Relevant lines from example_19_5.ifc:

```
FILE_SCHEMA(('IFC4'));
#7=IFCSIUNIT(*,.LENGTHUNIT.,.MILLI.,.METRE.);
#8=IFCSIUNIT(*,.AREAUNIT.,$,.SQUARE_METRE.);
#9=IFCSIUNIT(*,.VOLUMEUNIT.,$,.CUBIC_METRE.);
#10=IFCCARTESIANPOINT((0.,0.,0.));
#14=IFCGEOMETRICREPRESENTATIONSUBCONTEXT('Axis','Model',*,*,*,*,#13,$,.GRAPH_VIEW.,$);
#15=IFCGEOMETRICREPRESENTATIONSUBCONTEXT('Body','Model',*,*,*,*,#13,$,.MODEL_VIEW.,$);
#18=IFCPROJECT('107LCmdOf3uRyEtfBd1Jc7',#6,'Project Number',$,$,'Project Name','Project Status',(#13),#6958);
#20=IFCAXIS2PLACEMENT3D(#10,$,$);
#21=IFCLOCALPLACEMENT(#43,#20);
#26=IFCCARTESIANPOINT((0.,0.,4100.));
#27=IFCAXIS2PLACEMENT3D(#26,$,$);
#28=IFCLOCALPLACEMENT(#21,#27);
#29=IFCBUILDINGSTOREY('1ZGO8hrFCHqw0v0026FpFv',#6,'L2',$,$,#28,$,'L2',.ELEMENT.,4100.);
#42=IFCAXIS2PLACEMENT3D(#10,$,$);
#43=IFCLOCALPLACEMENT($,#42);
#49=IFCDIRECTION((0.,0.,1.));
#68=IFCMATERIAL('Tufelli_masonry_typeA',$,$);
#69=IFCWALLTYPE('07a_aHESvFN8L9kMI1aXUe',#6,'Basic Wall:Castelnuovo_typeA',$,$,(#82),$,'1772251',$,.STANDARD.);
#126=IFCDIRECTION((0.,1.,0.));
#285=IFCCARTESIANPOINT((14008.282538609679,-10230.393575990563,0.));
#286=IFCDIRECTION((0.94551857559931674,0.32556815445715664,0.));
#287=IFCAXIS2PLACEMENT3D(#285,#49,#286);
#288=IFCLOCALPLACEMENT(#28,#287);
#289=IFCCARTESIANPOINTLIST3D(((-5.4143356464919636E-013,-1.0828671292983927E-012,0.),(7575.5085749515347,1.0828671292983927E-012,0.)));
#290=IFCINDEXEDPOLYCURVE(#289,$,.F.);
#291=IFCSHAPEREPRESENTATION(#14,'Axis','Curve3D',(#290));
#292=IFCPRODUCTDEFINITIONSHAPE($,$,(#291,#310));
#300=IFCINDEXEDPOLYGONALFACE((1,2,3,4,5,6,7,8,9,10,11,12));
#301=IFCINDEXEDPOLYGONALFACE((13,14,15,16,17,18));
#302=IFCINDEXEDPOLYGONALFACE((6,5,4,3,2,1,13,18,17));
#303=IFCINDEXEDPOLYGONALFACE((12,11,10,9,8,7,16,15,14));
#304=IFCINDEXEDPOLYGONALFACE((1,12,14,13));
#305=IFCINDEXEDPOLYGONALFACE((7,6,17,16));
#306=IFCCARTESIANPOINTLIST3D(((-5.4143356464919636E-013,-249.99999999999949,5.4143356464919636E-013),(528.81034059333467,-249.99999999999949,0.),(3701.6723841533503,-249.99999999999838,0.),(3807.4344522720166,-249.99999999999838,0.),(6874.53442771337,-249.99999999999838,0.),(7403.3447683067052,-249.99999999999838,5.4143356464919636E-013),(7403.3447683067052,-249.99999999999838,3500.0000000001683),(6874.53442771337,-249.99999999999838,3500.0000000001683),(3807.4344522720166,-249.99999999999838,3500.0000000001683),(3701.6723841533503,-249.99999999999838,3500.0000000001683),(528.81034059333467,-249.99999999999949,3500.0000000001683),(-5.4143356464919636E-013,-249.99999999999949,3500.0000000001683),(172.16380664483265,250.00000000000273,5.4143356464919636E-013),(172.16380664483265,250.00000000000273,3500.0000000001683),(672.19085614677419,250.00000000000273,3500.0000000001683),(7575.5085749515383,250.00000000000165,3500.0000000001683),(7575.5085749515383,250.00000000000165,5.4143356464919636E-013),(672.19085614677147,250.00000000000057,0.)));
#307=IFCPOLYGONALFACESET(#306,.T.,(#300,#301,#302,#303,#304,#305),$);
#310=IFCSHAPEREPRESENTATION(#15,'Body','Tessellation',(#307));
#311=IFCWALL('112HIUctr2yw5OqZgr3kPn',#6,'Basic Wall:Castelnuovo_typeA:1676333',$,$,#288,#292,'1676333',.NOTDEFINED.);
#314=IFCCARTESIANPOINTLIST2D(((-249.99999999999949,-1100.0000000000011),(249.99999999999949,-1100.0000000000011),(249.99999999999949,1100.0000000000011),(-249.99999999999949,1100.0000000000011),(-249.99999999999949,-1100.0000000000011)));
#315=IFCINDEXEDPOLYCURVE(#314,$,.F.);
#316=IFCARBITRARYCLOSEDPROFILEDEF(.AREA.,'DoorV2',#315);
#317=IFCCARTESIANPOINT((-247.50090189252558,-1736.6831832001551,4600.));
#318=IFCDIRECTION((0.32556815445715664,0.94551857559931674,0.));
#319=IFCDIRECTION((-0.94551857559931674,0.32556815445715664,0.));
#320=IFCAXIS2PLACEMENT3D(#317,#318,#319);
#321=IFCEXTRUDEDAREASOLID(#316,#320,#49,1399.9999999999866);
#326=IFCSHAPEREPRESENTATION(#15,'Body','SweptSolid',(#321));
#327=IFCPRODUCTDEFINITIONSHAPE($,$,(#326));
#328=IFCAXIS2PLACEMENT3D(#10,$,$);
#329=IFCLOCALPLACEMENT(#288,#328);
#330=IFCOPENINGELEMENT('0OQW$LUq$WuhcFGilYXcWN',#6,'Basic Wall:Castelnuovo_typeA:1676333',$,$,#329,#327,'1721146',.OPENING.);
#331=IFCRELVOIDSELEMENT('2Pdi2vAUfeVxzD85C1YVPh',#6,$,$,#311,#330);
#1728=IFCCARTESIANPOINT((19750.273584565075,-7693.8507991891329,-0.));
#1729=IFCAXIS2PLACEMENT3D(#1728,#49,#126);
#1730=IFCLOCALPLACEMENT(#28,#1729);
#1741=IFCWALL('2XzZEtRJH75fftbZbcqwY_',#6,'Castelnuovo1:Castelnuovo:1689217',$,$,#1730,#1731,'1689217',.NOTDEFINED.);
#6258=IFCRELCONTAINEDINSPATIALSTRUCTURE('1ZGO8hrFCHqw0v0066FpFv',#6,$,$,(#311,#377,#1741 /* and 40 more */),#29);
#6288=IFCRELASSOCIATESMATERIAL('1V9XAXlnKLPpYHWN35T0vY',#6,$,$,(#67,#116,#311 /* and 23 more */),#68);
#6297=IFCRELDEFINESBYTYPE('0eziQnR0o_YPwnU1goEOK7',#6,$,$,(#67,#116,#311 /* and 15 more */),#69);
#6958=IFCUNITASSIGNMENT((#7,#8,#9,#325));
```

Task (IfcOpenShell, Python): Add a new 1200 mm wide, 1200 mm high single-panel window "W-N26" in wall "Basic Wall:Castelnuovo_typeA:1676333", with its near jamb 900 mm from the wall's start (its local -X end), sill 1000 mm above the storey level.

```python
import numpy as np
import ifcopenshell
import ifcopenshell.api.feature
import ifcopenshell.api.geometry
import ifcopenshell.api.root
import ifcopenshell.api.spatial
import ifcopenshell.geom
import ifcopenshell.util.element
import ifcopenshell.util.placement
import ifcopenshell.util.representation
import ifcopenshell.util.shape
import ifcopenshell.util.unit

model = ifcopenshell.open("example_19_5.ifc")
unit_scale = ifcopenshell.util.unit.calculate_unit_scale(model)
settings = ifcopenshell.geom.settings()


def volume(element):
    """Net volume in cubic metres, openings subtracted."""
    shape = ifcopenshell.geom.create_shape(settings, element)
    return ifcopenshell.util.shape.get_volume(shape.geometry)


wall = model.by_guid("112HIUctr2yw5OqZgr3kPn")
storey = ifcopenshell.util.element.get_container(wall, ifc_class="IfcBuildingStorey")
context = ifcopenshell.util.representation.get_context(model, "Model", "Body", "MODEL_VIEW")
before = volume(wall)

width, height, from_end, sill = 1.2, 1.2, 0.9, 1  # metres

# The wall runs along its own X axis, and the end named is its -X end.
wall_shape = ifcopenshell.geom.create_shape(settings, wall)
x, y, z = ifcopenshell.util.shape.get_vertices(wall_shape.geometry).T
start = x.min() + from_end
face, thickness = float(y.min()), float(y.max() - y.min())
wall_matrix = ifcopenshell.util.placement.get_local_placement(wall.ObjectPlacement)
level = ifcopenshell.util.placement.get_local_placement(storey.ObjectPlacement)[2, 3]


def in_wall(x, y):
    """Placement at x, y metres in the wall's axes, at sill height."""
    matrix = wall_matrix.copy()
    matrix[:, 3] = wall_matrix @ np.array([x / unit_scale, y / unit_scale, 0.0, 1.0])
    matrix[2, 3] = level + sill / unit_scale
    return matrix


# Opening: a box that overshoots both wall faces by 50 mm.
opening = ifcopenshell.api.root.create_entity(model, ifc_class="IfcOpeningElement", predefined_type="OPENING")
box = ifcopenshell.api.geometry.add_wall_representation(
    model, context=context, length=width, height=height, thickness=thickness + 0.1
)
ifcopenshell.api.geometry.assign_representation(model, product=opening, representation=box)
ifcopenshell.api.geometry.edit_object_placement(model, product=opening, matrix=in_wall(start, face - 0.05), is_si=False)
ifcopenshell.api.feature.add_feature(model, feature=opening, element=wall)

window = ifcopenshell.api.root.create_entity(model, ifc_class="IfcWindow", name="W-N26", predefined_type="WINDOW")
window.OverallWidth, window.OverallHeight = width / unit_scale, height / unit_scale
window.PartitioningType = "SINGLE_PANEL"
body = ifcopenshell.api.geometry.add_window_representation(
    model,
    context=context,
    overall_width=window.OverallWidth,
    overall_height=window.OverallHeight,
    partition_type="SINGLE_PANEL",
)
ifcopenshell.api.geometry.assign_representation(model, product=window, representation=body)
ifcopenshell.api.spatial.assign_container(model, products=[window], relating_structure=storey)
ifcopenshell.api.feature.add_filling(model, opening=opening, element=window)

# Centre the window in the wall's thickness.
ifcopenshell.api.geometry.edit_object_placement(model, product=window, matrix=in_wall(start, face), is_si=False)
window_shape = ifcopenshell.geom.create_shape(settings, window)
depth = ifcopenshell.util.shape.get_vertices(window_shape.geometry)[:, 1]
offset = face + thickness / 2 - (depth.min() + depth.max()) / 2
ifcopenshell.api.geometry.edit_object_placement(model, product=window, matrix=in_wall(start, offset), is_si=False)

after = volume(wall)

print(f"wall volume {before:.3f} -> {after:.3f} m3")

model.write("example_19_5_edited.ifc")
```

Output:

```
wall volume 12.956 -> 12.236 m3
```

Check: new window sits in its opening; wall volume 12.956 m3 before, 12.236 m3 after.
